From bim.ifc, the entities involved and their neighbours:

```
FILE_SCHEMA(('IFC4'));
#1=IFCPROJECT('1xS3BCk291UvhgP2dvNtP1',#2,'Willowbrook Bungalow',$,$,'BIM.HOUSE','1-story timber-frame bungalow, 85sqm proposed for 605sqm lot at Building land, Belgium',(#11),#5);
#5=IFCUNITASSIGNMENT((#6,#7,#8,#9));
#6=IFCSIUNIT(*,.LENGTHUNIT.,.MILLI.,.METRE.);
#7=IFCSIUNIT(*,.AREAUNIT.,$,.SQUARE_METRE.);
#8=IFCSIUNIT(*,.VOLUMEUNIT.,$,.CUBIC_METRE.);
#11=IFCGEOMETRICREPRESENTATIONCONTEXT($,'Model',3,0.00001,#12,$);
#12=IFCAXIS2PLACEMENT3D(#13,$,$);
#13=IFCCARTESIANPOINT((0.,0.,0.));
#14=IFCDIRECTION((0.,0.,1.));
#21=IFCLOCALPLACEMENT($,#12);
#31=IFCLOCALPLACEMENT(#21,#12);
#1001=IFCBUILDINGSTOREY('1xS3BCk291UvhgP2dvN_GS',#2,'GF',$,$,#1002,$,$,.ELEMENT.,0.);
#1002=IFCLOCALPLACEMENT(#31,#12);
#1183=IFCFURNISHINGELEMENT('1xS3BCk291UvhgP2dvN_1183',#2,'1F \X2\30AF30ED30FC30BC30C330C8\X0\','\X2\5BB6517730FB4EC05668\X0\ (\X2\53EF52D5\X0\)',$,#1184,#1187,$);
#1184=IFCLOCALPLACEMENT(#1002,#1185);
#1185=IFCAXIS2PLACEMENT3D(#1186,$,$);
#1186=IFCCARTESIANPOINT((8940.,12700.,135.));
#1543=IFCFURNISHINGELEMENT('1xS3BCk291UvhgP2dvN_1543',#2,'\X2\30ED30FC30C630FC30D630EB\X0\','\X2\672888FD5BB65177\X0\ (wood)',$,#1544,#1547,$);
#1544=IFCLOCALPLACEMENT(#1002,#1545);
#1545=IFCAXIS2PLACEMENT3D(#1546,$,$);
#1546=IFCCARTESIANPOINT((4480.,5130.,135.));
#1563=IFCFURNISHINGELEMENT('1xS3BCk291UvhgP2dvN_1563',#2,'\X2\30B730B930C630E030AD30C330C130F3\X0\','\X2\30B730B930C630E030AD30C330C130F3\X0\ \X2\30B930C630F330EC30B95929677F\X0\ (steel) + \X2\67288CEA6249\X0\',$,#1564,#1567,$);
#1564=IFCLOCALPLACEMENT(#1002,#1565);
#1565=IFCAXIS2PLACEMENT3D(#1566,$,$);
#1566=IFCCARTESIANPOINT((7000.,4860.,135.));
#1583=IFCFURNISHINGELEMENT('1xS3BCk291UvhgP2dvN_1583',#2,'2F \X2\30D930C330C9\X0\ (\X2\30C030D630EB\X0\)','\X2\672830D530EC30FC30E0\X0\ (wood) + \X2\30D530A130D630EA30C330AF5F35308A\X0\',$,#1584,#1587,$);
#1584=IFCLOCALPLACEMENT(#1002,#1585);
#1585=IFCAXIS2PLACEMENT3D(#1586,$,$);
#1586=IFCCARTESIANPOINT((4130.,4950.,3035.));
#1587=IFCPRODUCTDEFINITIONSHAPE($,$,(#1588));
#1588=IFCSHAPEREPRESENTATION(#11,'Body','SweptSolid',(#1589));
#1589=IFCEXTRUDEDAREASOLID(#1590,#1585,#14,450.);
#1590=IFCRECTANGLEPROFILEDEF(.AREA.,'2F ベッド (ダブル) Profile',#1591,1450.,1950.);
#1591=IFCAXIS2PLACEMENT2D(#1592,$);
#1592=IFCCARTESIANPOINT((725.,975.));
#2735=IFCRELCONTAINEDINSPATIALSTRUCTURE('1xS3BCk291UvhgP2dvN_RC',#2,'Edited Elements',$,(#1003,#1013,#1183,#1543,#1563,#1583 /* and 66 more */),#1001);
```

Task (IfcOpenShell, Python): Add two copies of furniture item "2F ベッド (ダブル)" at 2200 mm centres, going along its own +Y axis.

```python
import ifcopenshell
import ifcopenshell.api.geometry
import ifcopenshell.api.root
import ifcopenshell.util.element
import ifcopenshell.util.placement
import ifcopenshell.util.unit

model = ifcopenshell.open("bim.ifc")
unit_scale = ifcopenshell.util.unit.calculate_unit_scale(model)


def reuse_history(source, copy):
    """copy_class also copies each property set's owner history, people and application; keep the originals."""
    for rel in copy.IsDefinedBy:
        if rel.is_a("IfcRelDefinesByProperties") and (history := rel.RelatingPropertyDefinition.OwnerHistory):
            rel.RelatingPropertyDefinition.OwnerHistory = source.OwnerHistory
            ifcopenshell.util.element.remove_deep2(model, history)


source = model.by_guid("1xS3BCk291UvhgP2dvN_1583")
base = ifcopenshell.util.placement.get_local_placement(source.ObjectPlacement)
step = base[:3, 1] * 2.2 / unit_scale

for i in range(1, 3):
    copy = ifcopenshell.api.root.copy_class(model, product=source)
    copy.Representation = ifcopenshell.util.element.copy_deep(
        model, source.Representation, exclude=["IfcGeometricRepresentationContext", "IfcRepresentationMap"]
    )
    reuse_history(source, copy)
    matrix = base.copy()
    matrix[:3, 3] += i * step
    print("added at", matrix[:3, 3].round(3) + 0.0)
    ifcopenshell.api.geometry.edit_object_placement(model, product=copy, matrix=matrix, is_si=False)

model.write("bim_updated.ifc")
```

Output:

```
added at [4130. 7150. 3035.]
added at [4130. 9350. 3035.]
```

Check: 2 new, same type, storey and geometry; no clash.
